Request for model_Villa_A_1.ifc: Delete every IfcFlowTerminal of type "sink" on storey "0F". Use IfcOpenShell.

First a look at what the model holds.

```python
import ifcopenshell
import ifcopenshell.util.element

model = ifcopenshell.open("model_Villa_A_1.ifc")
print(model.schema)
storey = next(s for s in model.by_type("IfcBuildingStorey") if s.Name == "0F")
terminals = [e for e in ifcopenshell.util.element.get_decomposition(storey) if e.is_a("IfcFlowTerminal")]
seen = {}
for e in terminals:
    element_type = ifcopenshell.util.element.get_type(e)
    name = element_type.Name if element_type not in (None, e) else None
    seen[name] = seen.get(name, 0) + 1
for name, count in sorted(seen.items(), key=str):
    print(count, "x", name)
```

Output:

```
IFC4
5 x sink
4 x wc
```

```python
import ifcopenshell
import ifcopenshell.api.root
import ifcopenshell.util.element

model = ifcopenshell.open("model_Villa_A_1.ifc")

storey = next(s for s in model.by_type("IfcBuildingStorey") if s.Name == "0F")
terminals = [e for e in ifcopenshell.util.element.get_decomposition(storey) if e.is_a("IfcFlowTerminal")]
targets = [e for e in terminals if (t := ifcopenshell.util.element.get_type(e)) not in (None, e) and t.Name == "sink"]

for e in targets:
    ifcopenshell.api.root.remove_product(model, product=e)
print(len(targets), "removed")

model.write("model_Villa_A_1_v2.ifc")
```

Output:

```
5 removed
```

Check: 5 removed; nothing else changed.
